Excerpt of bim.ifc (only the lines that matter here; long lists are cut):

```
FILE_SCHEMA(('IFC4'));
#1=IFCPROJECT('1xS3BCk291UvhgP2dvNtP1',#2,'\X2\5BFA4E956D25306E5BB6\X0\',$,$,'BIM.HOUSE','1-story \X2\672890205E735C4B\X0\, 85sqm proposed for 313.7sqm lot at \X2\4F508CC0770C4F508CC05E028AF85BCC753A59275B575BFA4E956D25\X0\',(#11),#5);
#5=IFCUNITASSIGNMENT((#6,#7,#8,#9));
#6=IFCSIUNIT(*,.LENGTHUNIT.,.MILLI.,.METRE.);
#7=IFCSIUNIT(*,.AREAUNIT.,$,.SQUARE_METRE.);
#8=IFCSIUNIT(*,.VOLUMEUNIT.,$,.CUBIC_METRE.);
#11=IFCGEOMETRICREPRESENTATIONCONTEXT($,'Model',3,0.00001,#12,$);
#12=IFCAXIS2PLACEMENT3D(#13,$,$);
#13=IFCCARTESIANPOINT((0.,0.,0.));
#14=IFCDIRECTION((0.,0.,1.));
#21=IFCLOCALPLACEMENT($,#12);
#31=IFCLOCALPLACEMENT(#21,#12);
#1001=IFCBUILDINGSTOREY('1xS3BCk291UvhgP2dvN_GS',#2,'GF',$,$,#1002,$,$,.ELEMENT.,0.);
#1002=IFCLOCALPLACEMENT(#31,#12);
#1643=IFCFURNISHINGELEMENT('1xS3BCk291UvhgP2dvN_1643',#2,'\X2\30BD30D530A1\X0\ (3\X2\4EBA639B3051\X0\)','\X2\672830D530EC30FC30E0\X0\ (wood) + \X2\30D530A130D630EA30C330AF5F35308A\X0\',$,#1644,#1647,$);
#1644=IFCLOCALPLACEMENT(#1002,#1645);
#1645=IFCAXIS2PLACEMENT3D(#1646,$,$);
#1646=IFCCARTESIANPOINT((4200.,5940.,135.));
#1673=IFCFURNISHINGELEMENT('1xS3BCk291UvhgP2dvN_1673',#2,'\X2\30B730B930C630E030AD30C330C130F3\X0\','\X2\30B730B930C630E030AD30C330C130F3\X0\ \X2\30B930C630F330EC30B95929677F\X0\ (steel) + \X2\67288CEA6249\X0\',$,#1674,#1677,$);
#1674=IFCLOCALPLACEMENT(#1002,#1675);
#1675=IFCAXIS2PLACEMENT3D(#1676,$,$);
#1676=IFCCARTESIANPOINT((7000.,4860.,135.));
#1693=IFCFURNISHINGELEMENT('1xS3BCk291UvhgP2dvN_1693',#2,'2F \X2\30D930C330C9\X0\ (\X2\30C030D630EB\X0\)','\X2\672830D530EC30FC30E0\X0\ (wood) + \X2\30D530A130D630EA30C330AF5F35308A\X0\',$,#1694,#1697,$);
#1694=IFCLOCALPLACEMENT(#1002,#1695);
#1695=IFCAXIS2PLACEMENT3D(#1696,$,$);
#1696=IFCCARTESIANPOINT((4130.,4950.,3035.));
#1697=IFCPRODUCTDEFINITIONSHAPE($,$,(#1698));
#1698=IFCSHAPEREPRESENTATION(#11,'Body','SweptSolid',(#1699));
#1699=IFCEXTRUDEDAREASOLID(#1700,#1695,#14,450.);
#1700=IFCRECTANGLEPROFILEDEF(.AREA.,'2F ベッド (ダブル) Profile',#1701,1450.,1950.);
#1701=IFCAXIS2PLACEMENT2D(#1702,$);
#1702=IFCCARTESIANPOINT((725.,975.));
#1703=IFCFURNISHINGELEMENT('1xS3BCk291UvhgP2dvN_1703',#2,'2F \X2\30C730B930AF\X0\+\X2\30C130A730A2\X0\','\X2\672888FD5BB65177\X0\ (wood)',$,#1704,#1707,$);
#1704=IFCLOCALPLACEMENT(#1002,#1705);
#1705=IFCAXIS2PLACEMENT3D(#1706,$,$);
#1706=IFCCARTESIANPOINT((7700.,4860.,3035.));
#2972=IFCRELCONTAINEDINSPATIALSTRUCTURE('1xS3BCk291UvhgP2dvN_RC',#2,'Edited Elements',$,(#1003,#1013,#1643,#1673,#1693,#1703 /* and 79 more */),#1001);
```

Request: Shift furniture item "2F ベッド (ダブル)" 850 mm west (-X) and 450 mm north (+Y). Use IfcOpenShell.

```python
import ifcopenshell
import ifcopenshell.api.geometry
import ifcopenshell.util.placement
import ifcopenshell.util.unit

model = ifcopenshell.open("bim.ifc")
unit_scale = ifcopenshell.util.unit.calculate_unit_scale(model)

item = model.by_guid("1xS3BCk291UvhgP2dvN_1693")
matrix = ifcopenshell.util.placement.get_local_placement(item.ObjectPlacement)
matrix[0, 3] -= 0.85 / unit_scale
matrix[1, 3] += 0.45 / unit_scale
ifcopenshell.api.geometry.edit_object_placement(model, product=item, matrix=matrix, is_si=False)

print(ifcopenshell.util.placement.get_local_placement(item.ObjectPlacement).round(3) + 0.0)

model.write("bim_v2.ifc")
```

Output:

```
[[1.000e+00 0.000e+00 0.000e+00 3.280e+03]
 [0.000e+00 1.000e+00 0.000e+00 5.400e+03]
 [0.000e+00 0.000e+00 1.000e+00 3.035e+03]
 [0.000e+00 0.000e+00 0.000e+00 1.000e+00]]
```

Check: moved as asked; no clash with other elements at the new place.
